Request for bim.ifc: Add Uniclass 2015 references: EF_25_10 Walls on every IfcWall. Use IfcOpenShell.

First a look at what the model holds.

```python
import ifcopenshell

model = ifcopenshell.open("bim.ifc")
print(model.schema)
print("classifications:", [c.Name for c in model.by_type("IfcClassification")])
for ifc_class in ("IfcDoor", "IfcRoof", "IfcStair", "IfcWall", "IfcWindow"):
    print(ifc_class, len(model.by_type(ifc_class)))
```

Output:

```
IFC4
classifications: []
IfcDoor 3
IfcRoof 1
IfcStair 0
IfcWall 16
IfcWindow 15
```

```python
import ifcopenshell
import ifcopenshell.api.classification

model = ifcopenshell.open("bim.ifc")

system = ifcopenshell.api.classification.add_classification(model, classification="Uniclass 2015")

codes = {
    "IfcWall": ("EF_25_10", "Walls"),
}
for ifc_class, (code, name) in codes.items():
    products = model.by_type(ifc_class)
    ifcopenshell.api.classification.add_reference(
        model, products=products, classification=system, identification=code, name=name
    )
    print(code, len(products))

model.write("bim_rev.ifc")
```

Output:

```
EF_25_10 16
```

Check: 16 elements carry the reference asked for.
